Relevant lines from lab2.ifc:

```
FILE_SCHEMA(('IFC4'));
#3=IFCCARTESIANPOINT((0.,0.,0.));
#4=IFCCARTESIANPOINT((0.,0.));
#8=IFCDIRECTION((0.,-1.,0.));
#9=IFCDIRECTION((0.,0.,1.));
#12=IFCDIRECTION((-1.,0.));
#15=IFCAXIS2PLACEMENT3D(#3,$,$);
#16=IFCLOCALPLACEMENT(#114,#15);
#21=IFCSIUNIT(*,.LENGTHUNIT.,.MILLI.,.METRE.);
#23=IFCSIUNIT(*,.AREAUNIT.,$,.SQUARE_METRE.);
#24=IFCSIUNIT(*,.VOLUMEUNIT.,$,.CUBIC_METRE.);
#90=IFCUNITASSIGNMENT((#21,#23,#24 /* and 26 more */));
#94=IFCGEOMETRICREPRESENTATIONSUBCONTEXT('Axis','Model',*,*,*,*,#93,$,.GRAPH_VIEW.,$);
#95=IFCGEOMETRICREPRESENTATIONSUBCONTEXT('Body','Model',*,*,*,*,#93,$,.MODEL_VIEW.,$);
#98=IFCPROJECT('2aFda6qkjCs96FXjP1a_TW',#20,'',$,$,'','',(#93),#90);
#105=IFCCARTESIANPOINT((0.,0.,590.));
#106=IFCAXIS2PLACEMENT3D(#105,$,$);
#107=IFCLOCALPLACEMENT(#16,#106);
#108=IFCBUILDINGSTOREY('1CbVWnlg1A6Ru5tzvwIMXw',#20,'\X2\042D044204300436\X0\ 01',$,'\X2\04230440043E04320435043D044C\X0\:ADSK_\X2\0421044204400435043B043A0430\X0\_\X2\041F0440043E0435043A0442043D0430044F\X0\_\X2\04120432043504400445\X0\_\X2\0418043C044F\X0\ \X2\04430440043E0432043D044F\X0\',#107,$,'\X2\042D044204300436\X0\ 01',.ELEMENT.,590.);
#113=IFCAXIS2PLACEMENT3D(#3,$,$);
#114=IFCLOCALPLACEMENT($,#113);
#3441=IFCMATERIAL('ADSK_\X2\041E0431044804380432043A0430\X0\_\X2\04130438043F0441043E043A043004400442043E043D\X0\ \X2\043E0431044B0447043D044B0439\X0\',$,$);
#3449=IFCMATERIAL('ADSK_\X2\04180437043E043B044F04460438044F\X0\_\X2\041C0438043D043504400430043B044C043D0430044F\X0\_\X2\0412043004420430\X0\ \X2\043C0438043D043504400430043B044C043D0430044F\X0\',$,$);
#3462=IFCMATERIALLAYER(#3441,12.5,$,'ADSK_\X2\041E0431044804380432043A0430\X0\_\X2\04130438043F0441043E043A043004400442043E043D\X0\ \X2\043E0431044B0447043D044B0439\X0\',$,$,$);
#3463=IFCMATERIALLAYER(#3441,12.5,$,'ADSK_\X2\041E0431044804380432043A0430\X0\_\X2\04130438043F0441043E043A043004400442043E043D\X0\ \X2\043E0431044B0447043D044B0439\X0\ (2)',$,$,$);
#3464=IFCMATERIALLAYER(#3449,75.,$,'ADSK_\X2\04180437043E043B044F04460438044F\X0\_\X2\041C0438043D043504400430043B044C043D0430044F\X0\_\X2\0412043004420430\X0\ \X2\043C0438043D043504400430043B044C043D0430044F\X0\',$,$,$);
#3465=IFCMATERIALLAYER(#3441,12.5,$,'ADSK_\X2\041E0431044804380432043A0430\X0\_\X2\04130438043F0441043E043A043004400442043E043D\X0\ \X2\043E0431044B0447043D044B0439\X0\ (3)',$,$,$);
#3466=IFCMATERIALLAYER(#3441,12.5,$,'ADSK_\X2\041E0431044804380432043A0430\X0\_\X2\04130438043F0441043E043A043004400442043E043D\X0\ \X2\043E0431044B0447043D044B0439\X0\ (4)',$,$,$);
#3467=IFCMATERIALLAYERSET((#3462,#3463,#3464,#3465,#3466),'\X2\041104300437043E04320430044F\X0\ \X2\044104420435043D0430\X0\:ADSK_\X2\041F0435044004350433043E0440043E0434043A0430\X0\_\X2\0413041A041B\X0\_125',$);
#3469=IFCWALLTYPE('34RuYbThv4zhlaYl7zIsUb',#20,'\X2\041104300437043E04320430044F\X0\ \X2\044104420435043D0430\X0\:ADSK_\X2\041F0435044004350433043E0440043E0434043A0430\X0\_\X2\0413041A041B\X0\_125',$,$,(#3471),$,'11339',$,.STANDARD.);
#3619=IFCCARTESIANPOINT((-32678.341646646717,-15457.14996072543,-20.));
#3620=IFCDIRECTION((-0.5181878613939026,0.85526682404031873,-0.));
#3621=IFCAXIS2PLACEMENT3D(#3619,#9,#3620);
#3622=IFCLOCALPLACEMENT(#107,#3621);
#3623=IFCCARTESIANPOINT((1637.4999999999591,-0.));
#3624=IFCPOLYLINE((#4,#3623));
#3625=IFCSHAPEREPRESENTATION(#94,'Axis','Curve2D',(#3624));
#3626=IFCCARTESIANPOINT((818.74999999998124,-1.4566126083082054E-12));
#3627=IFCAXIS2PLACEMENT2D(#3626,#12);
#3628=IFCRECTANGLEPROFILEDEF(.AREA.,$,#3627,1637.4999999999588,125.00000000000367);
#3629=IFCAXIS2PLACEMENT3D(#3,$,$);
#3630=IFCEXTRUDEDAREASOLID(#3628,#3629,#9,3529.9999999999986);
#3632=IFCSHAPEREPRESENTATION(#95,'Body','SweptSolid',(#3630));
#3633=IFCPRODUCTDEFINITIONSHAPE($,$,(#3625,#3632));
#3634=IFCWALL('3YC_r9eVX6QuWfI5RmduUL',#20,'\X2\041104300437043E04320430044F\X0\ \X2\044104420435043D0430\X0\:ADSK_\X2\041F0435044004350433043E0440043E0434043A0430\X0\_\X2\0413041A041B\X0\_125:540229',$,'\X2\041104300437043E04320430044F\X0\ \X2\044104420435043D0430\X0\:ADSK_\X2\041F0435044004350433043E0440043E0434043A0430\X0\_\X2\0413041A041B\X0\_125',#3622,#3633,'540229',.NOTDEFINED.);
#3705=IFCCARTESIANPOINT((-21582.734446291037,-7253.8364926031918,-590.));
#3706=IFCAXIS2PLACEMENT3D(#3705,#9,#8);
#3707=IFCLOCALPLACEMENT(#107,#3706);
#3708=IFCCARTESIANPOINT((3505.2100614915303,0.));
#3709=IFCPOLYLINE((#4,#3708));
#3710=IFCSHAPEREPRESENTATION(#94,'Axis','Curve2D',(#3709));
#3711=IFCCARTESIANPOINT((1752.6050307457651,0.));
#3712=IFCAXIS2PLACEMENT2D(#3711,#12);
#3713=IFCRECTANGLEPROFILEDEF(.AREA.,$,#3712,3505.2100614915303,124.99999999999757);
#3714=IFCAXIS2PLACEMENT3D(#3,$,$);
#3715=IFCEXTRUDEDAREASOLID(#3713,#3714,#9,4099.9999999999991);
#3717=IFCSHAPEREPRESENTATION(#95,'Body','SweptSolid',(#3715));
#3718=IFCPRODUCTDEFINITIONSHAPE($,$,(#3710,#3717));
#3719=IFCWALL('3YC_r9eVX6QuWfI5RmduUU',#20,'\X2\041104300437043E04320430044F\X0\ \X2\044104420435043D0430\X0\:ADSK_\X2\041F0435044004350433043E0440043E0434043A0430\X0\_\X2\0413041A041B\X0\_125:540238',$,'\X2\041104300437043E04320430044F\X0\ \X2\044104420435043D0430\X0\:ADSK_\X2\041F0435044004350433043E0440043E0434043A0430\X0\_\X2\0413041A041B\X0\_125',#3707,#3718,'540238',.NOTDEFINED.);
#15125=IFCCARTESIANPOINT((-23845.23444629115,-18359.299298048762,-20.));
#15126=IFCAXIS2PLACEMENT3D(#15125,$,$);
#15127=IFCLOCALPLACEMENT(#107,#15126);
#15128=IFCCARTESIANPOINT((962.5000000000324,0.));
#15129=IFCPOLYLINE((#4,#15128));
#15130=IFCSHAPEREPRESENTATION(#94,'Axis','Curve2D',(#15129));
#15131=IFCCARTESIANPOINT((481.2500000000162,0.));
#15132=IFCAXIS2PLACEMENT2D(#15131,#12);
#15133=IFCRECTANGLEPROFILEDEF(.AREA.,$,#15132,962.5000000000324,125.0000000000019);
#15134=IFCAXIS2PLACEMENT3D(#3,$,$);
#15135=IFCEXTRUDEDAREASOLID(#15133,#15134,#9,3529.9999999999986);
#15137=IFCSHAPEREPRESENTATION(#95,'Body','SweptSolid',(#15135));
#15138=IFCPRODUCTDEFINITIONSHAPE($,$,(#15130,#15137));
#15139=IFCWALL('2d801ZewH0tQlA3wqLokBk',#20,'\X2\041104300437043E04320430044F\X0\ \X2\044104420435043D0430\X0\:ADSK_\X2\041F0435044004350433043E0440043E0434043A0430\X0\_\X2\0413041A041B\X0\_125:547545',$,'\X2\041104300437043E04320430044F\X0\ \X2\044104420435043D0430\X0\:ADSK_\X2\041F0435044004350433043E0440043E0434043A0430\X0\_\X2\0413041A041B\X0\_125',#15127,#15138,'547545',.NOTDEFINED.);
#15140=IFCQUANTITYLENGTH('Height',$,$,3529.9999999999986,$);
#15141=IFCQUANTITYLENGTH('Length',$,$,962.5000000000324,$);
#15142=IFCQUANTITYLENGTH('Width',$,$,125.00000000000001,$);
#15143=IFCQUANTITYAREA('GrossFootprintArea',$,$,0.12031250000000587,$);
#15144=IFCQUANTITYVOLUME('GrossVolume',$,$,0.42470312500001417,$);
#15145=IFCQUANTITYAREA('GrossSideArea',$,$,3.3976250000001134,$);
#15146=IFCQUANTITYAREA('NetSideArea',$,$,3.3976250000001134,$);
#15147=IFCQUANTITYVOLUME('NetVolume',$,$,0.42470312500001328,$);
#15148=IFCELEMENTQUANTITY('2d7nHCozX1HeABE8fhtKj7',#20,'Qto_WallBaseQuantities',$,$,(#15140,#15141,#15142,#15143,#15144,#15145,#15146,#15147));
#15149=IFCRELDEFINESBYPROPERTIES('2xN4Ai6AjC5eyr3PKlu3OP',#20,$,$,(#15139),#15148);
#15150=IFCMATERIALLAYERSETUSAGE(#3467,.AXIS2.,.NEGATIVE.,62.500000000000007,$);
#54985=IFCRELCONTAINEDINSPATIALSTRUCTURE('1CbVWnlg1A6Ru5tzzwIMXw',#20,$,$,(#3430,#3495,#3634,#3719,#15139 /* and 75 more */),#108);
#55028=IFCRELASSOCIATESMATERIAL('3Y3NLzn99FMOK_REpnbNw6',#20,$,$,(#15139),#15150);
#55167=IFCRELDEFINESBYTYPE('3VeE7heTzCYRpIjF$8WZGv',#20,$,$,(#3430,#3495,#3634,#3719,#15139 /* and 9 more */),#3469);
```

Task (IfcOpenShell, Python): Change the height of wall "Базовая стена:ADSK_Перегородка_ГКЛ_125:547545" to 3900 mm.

```python
import ifcopenshell
import ifcopenshell.api.pset
import ifcopenshell.geom
import ifcopenshell.util.element
import ifcopenshell.util.representation
import ifcopenshell.util.shape
import ifcopenshell.util.unit

model = ifcopenshell.open("lab2.ifc")
unit_scale = ifcopenshell.util.unit.calculate_unit_scale(model)
area_scale = ifcopenshell.util.unit.calculate_unit_scale(model, "AREAUNIT")
volume_scale = ifcopenshell.util.unit.calculate_unit_scale(model, "VOLUMEUNIT")
settings = ifcopenshell.geom.settings()


def volume(element):
    """Net volume in cubic metres, openings subtracted."""
    shape = ifcopenshell.geom.create_shape(settings, element)
    return ifcopenshell.util.shape.get_volume(shape.geometry)


wall = model.by_guid("2d801ZewH0tQlA3wqLokBk")
before = volume(wall)

body = ifcopenshell.util.representation.get_representation(wall, "Model", "Body")
solid = body.Items[0]
old_height = solid.Depth
solid.Depth = 3900.0
after = volume(wall)
thickness = 0.125  # wall thickness in metres

# Update the stored height, areas and volumes.
qto = model.by_id(ifcopenshell.util.element.get_pset(wall, "Qto_WallBaseQuantities", should_inherit=False)["id"])
ifcopenshell.api.pset.edit_qto(model, qto=qto, properties={
    "Height": solid.Depth,
    "GrossVolume": ifcopenshell.util.element.get_pset(wall, "Qto_WallBaseQuantities", "GrossVolume") * solid.Depth / old_height,
    "GrossSideArea": ifcopenshell.util.element.get_pset(wall, "Qto_WallBaseQuantities", "GrossSideArea") * solid.Depth / old_height,
    "NetSideArea": after / thickness / area_scale,
    "NetVolume": after / volume_scale,
})

print(f"height {old_height:g} -> {solid.Depth:g}, volume {before:.3f} -> {after:.3f} m3")

model.write("lab2_updated.ifc")
```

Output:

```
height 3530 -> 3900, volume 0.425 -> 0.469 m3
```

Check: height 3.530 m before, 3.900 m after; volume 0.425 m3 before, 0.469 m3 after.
